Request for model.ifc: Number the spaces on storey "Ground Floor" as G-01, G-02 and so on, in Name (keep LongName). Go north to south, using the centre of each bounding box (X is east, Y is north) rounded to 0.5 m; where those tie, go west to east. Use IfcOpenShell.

First a look at what the model holds.

```python
import ifcopenshell
import ifcopenshell.util.element
import ifcopenshell.util.placement

model = ifcopenshell.open("model.ifc")
print(model.schema)
storey = next(s for s in model.by_type("IfcBuildingStorey") if s.Name == "Ground Floor")
spaces = [e for e in ifcopenshell.util.element.get_decomposition(storey) if e.is_a("IfcSpace")]
for e in sorted(spaces, key=lambda e: e.id()):
    origin = ifcopenshell.util.placement.get_local_placement(e.ObjectPlacement)[:3, 3]
    print(e.id(), e.Name, e.LongName, origin.round(2) + 0.0, sep=" | ")
```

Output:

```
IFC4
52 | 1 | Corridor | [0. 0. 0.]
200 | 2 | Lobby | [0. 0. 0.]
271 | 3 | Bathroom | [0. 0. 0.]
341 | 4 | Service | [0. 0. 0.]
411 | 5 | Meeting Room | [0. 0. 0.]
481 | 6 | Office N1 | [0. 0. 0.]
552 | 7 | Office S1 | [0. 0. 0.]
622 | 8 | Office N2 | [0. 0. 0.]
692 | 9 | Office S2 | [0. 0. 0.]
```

```python
import ifcopenshell
import ifcopenshell.geom
import ifcopenshell.util.element
import ifcopenshell.util.shape

model = ifcopenshell.open("model.ifc")
settings = ifcopenshell.geom.settings()
settings.set("use-world-coords", True)


def centre(element):
    shape = ifcopenshell.geom.create_shape(settings, element)
    return ifcopenshell.util.shape.get_bbox_centroid(shape.geometry)


storey = next(s for s in model.by_type("IfcBuildingStorey") if s.Name == "Ground Floor")
spaces = [e for e in ifcopenshell.util.element.get_decomposition(storey) if e.is_a("IfcSpace")]

# Insertion points can sit at a corner or the storey origin, so sort by the geometry (in metres).
centres = {e: centre(e) for e in spaces}
spaces.sort(key=lambda e: (-round(centres[e][1] / 0.5), centres[e][0]))

for i, e in enumerate(spaces, start=1):
    number = f"G-{i:02d}"
    e.Name = number
    print(e.id(), number)

model.write("model-out.ifc")
```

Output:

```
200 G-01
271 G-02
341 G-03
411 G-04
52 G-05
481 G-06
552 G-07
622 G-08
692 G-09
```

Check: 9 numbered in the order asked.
